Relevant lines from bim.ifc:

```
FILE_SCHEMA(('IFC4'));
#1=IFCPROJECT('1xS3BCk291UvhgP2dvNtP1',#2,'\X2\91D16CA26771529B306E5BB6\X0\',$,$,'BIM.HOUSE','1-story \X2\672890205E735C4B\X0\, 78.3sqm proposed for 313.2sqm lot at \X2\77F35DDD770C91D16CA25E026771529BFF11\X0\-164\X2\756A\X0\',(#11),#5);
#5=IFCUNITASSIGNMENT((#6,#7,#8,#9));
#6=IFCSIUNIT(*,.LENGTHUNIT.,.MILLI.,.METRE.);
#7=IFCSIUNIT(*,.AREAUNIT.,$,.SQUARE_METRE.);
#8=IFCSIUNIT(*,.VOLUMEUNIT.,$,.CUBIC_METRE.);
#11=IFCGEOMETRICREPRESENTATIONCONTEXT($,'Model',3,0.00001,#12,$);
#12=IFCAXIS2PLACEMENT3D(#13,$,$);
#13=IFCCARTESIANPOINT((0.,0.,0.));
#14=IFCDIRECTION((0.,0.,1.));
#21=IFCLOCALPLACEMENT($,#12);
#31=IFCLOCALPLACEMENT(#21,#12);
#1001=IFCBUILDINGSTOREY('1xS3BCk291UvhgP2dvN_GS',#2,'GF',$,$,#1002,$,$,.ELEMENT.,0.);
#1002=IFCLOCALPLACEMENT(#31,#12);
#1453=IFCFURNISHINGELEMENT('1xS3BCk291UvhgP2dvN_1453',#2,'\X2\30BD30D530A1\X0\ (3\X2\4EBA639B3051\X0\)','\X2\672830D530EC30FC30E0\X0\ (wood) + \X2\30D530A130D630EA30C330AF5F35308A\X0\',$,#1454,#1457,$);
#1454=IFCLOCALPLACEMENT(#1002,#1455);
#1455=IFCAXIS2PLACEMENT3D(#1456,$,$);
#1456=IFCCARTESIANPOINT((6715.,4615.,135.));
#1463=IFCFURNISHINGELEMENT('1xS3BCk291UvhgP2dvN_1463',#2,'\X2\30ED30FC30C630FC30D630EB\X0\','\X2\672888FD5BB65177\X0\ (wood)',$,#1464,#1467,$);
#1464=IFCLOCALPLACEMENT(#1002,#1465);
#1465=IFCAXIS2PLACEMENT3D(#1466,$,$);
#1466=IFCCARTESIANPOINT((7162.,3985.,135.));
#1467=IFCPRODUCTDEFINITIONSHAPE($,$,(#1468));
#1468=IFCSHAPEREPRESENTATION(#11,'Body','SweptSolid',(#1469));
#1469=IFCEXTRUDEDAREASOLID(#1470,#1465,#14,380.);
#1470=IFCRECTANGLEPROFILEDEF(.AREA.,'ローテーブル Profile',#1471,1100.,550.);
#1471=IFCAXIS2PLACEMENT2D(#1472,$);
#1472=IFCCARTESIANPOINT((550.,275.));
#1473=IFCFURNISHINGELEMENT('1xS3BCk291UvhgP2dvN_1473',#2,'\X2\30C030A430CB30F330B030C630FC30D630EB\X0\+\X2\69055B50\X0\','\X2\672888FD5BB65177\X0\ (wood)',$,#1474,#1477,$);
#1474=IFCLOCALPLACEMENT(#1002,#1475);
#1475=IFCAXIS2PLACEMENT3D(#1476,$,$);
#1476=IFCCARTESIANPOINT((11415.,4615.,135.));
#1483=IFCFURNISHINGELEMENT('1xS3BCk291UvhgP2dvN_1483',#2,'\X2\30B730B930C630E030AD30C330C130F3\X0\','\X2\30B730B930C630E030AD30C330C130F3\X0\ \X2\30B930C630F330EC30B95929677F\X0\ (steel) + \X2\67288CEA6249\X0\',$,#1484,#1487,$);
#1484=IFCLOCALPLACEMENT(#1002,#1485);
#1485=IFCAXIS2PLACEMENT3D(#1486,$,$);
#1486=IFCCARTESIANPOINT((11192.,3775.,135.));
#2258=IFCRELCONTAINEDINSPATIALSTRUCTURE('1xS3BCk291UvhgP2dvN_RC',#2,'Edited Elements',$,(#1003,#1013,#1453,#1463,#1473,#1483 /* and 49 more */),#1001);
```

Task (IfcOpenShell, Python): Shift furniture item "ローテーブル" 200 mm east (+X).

```python
import ifcopenshell
import ifcopenshell.api.geometry
import ifcopenshell.util.placement
import ifcopenshell.util.unit

model = ifcopenshell.open("bim.ifc")
unit_scale = ifcopenshell.util.unit.calculate_unit_scale(model)

item = model.by_guid("1xS3BCk291UvhgP2dvN_1463")
matrix = ifcopenshell.util.placement.get_local_placement(item.ObjectPlacement)
matrix[0, 3] += 0.2 / unit_scale
ifcopenshell.api.geometry.edit_object_placement(model, product=item, matrix=matrix, is_si=False)

print(ifcopenshell.util.placement.get_local_placement(item.ObjectPlacement).round(3) + 0.0)

model.write("bim-out.ifc")
```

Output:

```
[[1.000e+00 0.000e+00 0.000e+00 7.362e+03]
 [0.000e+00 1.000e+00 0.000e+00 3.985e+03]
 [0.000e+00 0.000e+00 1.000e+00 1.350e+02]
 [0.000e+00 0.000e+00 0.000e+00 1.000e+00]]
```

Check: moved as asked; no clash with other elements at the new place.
